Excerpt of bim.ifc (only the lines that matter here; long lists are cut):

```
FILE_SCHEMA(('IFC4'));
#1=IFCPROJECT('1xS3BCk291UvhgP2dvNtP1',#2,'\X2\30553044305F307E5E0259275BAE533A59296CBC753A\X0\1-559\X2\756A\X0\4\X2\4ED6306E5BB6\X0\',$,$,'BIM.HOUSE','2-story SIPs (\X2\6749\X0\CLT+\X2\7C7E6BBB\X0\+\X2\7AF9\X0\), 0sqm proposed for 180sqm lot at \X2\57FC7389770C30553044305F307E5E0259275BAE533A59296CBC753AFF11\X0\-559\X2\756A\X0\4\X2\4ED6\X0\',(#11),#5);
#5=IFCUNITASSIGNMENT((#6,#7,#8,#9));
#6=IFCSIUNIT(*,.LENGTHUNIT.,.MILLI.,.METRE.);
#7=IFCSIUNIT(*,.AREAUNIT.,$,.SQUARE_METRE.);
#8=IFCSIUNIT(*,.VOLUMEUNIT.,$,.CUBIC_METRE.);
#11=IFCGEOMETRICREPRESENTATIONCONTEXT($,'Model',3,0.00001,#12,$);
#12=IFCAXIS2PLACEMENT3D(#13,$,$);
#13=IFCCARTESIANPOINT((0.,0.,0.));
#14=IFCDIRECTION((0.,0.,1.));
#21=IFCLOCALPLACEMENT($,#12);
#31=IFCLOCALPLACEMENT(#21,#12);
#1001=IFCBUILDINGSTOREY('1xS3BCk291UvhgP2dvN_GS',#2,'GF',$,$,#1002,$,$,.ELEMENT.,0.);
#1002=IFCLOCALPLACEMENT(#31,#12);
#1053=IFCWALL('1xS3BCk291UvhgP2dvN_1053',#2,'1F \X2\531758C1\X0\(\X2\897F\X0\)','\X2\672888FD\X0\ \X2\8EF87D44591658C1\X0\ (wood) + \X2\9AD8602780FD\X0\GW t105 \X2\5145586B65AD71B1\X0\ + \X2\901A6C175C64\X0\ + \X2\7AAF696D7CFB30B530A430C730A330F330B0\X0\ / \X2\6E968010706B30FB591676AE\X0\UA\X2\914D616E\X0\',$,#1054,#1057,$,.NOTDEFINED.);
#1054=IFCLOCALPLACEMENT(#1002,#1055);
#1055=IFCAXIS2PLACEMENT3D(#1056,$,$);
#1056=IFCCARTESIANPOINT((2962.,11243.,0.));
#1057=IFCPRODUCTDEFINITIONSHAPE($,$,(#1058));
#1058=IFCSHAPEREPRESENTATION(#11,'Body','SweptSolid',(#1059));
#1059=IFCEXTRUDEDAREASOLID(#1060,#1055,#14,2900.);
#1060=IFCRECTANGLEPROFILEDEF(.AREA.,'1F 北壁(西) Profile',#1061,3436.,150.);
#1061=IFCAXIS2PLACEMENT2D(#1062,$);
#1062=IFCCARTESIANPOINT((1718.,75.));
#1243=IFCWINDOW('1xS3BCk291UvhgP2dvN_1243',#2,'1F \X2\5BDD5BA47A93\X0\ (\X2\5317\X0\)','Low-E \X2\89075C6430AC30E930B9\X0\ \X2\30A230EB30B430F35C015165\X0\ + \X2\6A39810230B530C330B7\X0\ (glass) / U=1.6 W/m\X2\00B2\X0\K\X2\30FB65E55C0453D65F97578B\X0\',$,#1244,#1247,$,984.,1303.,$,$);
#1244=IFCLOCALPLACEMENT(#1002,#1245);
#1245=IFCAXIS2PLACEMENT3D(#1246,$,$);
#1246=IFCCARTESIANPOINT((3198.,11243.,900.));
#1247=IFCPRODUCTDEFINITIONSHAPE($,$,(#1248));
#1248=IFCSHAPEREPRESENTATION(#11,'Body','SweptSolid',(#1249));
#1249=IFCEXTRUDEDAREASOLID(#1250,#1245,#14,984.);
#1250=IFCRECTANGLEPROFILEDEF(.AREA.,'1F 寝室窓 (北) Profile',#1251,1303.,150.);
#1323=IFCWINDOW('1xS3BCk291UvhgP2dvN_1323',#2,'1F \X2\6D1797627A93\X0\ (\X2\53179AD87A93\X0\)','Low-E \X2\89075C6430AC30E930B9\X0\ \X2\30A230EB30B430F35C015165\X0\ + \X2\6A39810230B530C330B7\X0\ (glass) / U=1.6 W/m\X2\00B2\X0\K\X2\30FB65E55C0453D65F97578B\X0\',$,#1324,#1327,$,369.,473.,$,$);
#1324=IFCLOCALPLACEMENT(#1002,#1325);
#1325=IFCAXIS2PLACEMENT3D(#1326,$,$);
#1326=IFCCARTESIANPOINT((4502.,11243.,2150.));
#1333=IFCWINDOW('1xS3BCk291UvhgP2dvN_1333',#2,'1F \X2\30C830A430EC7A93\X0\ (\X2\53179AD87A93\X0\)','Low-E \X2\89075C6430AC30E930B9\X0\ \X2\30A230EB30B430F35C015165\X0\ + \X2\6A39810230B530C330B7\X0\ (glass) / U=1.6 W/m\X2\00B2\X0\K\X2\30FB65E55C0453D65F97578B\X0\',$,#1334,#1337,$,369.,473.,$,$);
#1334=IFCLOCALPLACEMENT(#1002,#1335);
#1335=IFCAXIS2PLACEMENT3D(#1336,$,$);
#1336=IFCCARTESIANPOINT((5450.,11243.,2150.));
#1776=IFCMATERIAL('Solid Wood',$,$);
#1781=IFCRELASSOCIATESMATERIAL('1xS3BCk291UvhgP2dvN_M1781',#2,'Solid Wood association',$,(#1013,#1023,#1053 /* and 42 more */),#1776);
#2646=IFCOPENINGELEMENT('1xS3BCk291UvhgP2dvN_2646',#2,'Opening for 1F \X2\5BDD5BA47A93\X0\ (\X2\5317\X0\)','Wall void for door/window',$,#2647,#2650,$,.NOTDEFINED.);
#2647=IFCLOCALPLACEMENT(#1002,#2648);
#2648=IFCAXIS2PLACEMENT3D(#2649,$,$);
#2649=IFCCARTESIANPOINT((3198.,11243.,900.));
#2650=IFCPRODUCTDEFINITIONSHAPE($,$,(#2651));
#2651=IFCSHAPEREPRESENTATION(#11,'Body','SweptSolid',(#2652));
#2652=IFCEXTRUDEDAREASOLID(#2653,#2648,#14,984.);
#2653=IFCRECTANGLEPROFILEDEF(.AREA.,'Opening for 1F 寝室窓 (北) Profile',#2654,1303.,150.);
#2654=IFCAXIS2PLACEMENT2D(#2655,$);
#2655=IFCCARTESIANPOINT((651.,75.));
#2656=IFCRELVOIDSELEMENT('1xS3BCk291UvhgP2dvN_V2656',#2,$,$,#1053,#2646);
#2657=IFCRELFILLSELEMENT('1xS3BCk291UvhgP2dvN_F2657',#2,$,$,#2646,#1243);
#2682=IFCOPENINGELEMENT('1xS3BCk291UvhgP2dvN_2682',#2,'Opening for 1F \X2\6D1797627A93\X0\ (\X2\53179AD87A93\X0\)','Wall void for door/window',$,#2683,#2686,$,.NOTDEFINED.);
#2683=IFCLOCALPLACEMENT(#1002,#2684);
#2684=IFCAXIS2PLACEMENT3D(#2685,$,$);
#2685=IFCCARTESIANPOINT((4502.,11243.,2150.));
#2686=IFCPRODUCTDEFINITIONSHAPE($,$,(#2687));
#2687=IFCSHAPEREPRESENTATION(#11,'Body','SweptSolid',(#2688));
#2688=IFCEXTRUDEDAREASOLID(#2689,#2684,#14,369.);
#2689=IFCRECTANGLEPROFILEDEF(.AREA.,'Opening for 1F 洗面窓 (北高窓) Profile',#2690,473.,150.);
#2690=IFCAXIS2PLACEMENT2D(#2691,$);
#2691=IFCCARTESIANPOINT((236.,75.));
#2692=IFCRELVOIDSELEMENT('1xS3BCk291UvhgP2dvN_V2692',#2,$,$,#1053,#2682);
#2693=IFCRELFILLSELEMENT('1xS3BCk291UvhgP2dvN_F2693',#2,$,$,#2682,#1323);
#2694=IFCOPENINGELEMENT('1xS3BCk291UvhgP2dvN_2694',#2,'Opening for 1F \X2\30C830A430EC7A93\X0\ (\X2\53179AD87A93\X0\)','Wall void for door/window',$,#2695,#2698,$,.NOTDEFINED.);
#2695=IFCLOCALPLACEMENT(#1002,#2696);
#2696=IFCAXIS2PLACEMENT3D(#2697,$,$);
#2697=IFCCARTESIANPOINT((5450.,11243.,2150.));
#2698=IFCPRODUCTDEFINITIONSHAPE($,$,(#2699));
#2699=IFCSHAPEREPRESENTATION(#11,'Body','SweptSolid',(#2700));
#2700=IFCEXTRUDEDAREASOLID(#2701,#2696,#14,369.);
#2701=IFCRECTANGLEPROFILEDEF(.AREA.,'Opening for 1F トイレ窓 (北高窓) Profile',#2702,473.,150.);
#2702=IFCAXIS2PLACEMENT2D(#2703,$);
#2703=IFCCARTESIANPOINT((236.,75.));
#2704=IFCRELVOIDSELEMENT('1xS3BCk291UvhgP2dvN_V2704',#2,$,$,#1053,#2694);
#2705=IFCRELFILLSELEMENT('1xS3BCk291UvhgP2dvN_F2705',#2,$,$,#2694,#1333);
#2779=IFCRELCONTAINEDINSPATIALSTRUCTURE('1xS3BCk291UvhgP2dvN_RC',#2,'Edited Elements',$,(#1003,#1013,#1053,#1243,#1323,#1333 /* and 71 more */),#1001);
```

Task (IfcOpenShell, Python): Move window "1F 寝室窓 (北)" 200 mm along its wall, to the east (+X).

```python
import ifcopenshell
import ifcopenshell.api.geometry
import ifcopenshell.util.placement
import ifcopenshell.util.unit

model = ifcopenshell.open("bim.ifc")
unit_scale = ifcopenshell.util.unit.calculate_unit_scale(model)

window = model.by_guid("1xS3BCk291UvhgP2dvN_1243")
opening = window.FillsVoids[0].RelatingOpeningElement
wall = opening.VoidsElements[0].RelatingBuildingElement

wall_matrix = ifcopenshell.util.placement.get_local_placement(wall.ObjectPlacement)
shift = wall_matrix[:3, 0] * 0.2 / unit_scale
before = ifcopenshell.util.placement.get_local_placement(window.ObjectPlacement)[:3, 3].copy()

# The window is not placed relative to its opening, so move both.
for product in (opening, window):
    matrix = ifcopenshell.util.placement.get_local_placement(product.ObjectPlacement)
    matrix[:3, 3] += shift
    ifcopenshell.api.geometry.edit_object_placement(model, product=product, matrix=matrix, is_si=False)

after = ifcopenshell.util.placement.get_local_placement(window.ObjectPlacement)[:3, 3]
print("window moved by", (after - before).round(3) + 0.0)

model.write("bim_rev.ifc")
```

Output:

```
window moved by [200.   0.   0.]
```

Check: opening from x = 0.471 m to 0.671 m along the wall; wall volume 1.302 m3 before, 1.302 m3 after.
